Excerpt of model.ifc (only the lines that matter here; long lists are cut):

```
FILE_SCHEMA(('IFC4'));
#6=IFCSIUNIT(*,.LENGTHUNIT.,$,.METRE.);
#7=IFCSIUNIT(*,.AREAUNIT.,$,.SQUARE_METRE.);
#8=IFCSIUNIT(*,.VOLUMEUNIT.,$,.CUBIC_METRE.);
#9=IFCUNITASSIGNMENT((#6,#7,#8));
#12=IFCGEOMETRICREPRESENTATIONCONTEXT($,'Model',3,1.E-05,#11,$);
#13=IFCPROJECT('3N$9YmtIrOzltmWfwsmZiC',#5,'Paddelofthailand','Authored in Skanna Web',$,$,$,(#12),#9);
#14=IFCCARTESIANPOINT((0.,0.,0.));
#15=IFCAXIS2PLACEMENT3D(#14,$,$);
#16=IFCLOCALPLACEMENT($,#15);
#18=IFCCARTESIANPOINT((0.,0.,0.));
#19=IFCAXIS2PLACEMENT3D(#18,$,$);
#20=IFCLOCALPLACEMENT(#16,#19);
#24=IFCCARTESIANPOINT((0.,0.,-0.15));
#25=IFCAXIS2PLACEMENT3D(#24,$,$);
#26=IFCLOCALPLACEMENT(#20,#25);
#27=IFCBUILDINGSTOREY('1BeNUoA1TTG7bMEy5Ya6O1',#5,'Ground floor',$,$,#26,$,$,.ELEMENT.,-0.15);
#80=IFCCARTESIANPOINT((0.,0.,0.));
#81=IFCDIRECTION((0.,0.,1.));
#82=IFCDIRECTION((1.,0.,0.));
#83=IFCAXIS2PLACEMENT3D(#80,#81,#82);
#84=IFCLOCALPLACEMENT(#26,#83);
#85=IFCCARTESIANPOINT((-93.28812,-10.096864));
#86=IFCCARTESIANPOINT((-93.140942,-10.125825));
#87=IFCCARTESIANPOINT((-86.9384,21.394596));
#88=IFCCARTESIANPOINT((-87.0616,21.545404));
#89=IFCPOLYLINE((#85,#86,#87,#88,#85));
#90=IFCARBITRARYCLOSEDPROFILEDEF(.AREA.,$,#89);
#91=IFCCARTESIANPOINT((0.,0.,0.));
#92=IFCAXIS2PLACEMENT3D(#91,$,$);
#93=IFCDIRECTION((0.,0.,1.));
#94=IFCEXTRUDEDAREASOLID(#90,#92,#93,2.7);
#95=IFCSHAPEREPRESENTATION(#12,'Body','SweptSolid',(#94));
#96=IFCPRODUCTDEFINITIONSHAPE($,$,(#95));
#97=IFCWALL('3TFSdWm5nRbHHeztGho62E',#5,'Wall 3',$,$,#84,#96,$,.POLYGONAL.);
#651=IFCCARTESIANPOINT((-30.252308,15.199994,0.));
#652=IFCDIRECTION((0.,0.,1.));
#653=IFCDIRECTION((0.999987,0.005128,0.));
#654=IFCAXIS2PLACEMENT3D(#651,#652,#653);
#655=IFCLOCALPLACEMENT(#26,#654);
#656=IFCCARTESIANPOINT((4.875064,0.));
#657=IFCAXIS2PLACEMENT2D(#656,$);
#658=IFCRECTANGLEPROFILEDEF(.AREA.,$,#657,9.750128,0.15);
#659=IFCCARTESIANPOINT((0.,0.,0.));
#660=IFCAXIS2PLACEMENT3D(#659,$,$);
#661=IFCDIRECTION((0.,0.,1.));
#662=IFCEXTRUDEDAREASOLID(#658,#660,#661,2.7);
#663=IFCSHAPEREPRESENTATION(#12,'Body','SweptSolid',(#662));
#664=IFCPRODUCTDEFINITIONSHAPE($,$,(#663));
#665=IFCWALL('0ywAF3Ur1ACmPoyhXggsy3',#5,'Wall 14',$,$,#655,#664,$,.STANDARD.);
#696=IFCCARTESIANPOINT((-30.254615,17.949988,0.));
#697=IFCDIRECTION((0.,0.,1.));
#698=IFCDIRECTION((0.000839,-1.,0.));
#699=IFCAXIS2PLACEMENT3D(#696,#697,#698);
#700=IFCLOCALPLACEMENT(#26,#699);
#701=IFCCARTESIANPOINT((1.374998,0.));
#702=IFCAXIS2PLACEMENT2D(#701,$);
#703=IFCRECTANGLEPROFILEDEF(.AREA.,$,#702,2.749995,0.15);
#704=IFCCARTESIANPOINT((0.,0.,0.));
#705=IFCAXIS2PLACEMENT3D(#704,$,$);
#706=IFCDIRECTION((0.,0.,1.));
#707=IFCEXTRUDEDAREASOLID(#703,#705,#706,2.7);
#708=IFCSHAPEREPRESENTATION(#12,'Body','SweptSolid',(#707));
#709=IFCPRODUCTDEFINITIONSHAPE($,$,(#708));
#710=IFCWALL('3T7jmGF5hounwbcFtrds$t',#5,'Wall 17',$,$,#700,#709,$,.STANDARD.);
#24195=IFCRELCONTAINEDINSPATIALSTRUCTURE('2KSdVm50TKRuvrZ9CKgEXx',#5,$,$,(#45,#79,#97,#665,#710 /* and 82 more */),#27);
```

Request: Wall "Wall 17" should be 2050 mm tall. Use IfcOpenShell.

```python
import ifcopenshell
import ifcopenshell.geom
import ifcopenshell.util.shape
import ifcopenshell.util.unit

model = ifcopenshell.open("model.ifc")
unit_scale = ifcopenshell.util.unit.calculate_unit_scale(model)
settings = ifcopenshell.geom.settings()


def volume(element):
    """Net volume in cubic metres, openings subtracted."""
    shape = ifcopenshell.geom.create_shape(settings, element)
    return ifcopenshell.util.shape.get_volume(shape.geometry)


wall = model.by_guid("3T7jmGF5hounwbcFtrds$t")
before = volume(wall)

body = next(r for r in wall.Representation.Representations if r.RepresentationIdentifier == "Body")
solid = body.Items[0]
old_height = solid.Depth
solid.Depth = 2.05 / unit_scale
after = volume(wall)

print(f"height {old_height:g} -> {solid.Depth:g}, volume {before:.3f} -> {after:.3f} m3")

model.write("model_updated.ifc")
```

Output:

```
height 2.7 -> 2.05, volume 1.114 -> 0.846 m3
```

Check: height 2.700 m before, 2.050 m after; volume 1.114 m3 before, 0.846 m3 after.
